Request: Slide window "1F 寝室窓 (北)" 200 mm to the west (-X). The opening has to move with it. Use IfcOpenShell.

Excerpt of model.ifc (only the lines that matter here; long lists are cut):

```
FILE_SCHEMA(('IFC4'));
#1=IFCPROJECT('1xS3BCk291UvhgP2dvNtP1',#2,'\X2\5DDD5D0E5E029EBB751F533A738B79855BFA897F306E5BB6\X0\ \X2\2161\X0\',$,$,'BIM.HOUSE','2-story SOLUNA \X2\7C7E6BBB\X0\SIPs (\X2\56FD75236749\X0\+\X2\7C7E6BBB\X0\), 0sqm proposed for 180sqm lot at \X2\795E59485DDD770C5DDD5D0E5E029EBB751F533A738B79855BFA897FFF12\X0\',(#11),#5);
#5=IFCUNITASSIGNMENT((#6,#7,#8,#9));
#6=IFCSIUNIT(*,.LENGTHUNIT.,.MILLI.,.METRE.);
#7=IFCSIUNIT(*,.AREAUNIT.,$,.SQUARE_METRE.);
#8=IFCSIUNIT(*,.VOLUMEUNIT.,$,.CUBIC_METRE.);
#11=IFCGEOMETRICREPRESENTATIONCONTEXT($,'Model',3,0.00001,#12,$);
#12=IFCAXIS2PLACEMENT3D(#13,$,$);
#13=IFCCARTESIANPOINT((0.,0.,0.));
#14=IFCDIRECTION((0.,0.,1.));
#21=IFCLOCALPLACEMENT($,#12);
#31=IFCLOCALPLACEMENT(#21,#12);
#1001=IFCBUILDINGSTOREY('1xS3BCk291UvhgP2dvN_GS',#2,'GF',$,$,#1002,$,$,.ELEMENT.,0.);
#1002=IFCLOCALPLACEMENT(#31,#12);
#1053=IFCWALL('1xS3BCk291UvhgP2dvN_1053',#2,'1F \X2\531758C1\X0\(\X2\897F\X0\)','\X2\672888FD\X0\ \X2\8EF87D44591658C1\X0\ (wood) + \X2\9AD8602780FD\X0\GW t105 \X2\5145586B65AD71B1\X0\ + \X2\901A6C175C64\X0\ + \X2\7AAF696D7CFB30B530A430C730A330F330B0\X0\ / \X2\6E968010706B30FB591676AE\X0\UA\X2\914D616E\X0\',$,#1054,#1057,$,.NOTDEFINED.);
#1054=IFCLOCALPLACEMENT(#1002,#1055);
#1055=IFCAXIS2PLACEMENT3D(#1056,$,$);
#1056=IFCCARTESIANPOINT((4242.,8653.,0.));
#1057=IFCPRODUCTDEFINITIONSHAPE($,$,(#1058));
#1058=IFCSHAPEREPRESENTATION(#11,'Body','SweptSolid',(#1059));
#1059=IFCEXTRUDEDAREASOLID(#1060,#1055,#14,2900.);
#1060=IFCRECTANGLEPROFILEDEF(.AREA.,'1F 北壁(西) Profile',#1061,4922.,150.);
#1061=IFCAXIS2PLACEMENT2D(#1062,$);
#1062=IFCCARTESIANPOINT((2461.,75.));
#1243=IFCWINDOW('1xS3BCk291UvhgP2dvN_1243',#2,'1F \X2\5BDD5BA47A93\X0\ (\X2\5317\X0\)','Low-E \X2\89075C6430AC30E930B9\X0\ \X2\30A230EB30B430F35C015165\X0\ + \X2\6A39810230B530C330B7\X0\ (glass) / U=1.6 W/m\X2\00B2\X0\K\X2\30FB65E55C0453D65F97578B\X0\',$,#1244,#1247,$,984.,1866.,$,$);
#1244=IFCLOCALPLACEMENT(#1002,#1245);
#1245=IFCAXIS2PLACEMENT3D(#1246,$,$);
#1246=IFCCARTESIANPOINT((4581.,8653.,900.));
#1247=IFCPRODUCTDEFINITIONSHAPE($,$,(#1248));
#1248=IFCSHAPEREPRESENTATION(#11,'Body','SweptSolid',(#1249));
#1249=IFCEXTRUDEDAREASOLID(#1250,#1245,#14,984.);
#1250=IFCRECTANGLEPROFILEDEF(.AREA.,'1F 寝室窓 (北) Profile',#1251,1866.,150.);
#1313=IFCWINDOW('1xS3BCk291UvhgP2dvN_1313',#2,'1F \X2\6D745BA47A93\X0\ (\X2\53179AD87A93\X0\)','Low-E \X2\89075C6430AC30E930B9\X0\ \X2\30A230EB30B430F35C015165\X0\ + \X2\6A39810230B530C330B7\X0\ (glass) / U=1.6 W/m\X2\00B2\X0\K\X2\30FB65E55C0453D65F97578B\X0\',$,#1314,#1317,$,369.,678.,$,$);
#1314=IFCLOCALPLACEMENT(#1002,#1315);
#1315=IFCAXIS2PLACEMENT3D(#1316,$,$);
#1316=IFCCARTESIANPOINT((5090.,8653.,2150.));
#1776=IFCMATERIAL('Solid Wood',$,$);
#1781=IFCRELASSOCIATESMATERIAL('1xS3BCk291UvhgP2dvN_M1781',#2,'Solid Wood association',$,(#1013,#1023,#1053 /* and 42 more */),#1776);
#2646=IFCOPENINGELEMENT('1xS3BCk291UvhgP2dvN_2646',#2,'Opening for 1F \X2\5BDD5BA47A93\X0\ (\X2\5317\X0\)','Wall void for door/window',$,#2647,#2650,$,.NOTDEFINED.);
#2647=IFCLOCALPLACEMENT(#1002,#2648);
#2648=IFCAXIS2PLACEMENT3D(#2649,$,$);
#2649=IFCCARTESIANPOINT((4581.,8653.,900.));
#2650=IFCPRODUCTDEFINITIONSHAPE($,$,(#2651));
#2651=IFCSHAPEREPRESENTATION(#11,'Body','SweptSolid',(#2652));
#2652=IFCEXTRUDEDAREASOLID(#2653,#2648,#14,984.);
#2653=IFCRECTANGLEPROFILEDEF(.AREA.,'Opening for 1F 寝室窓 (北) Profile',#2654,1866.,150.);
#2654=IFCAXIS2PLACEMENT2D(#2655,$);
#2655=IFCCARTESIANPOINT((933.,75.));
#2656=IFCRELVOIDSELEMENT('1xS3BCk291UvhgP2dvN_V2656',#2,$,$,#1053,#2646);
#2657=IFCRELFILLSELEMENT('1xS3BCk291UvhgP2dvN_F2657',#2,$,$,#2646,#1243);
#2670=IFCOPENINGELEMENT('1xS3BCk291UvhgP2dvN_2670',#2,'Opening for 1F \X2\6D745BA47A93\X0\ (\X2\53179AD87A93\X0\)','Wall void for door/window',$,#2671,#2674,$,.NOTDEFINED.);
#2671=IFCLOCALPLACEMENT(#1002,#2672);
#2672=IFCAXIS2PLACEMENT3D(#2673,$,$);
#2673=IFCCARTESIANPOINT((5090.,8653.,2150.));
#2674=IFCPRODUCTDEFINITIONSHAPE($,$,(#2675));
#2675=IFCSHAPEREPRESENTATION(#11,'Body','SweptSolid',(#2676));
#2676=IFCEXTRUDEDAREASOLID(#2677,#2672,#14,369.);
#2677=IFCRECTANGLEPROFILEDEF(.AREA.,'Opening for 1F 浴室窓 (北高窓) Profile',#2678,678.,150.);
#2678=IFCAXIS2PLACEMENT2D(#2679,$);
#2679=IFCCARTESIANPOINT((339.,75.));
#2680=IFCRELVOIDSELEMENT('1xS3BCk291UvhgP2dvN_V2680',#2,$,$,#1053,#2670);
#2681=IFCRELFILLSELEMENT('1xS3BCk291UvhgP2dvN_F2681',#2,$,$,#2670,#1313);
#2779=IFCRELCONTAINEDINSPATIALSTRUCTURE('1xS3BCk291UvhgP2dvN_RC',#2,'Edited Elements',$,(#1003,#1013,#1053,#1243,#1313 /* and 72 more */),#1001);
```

```python
import ifcopenshell
import ifcopenshell.api.geometry
import ifcopenshell.util.placement
import ifcopenshell.util.unit

model = ifcopenshell.open("model.ifc")
unit_scale = ifcopenshell.util.unit.calculate_unit_scale(model)

window = model.by_guid("1xS3BCk291UvhgP2dvN_1243")
opening = window.FillsVoids[0].RelatingOpeningElement
wall = opening.VoidsElements[0].RelatingBuildingElement

wall_matrix = ifcopenshell.util.placement.get_local_placement(wall.ObjectPlacement)
shift = wall_matrix[:3, 0] * -0.2 / unit_scale
before = ifcopenshell.util.placement.get_local_placement(window.ObjectPlacement)[:3, 3].copy()

# The window is not placed relative to its opening, so move both.
for product in (opening, window):
    matrix = ifcopenshell.util.placement.get_local_placement(product.ObjectPlacement)
    matrix[:3, 3] += shift
    ifcopenshell.api.geometry.edit_object_placement(model, product=product, matrix=matrix, is_si=False)

after = ifcopenshell.util.placement.get_local_placement(window.ObjectPlacement)[:3, 3]
print("window moved by", (after - before).round(3) + 0.0)

model.write("model_rev.ifc")
```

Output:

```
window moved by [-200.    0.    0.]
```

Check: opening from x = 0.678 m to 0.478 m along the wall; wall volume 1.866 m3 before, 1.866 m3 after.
